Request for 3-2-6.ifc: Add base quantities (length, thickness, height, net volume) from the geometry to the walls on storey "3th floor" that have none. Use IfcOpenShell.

First a look at what the model holds.

```python
import ifcopenshell
import ifcopenshell.util.element
import ifcopenshell.util.unit

model = ifcopenshell.open("3-2-6.ifc")
print(model.schema)
for unit_type in ("LENGTHUNIT", "AREAUNIT", "VOLUMEUNIT"):
    print(unit_type, ifcopenshell.util.unit.calculate_unit_scale(model, unit_type))
storey = next(s for s in model.by_type("IfcBuildingStorey") if s.Name == "3th floor")
walls = [e for e in ifcopenshell.util.element.get_decomposition(storey) if e.is_a("IfcWall")]
for e in sorted(walls, key=lambda e: e.id()):
    print(e.id(), e.is_a(), e.Name, list(ifcopenshell.util.element.get_psets(e, qtos_only=True)), sep=" | ")
```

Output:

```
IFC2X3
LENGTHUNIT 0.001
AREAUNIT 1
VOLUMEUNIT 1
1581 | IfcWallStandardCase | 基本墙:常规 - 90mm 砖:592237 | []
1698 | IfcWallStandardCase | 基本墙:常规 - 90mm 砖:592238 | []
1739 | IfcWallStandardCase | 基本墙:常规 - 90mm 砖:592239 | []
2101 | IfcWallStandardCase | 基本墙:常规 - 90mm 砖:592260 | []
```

```python
import ifcopenshell
import ifcopenshell.api.pset
import ifcopenshell.geom
import ifcopenshell.util.element
import ifcopenshell.util.shape
import ifcopenshell.util.unit

model = ifcopenshell.open("3-2-6.ifc")
unit_scale = ifcopenshell.util.unit.calculate_unit_scale(model)
volume_scale = ifcopenshell.util.unit.calculate_unit_scale(model, "VOLUMEUNIT")
settings = ifcopenshell.geom.settings()

storey = next(s for s in model.by_type("IfcBuildingStorey") if s.Name == "3th floor")
walls = [e for e in ifcopenshell.util.element.get_decomposition(storey) if e.is_a("IfcWall")]

for e in sorted(walls, key=lambda e: e.id()):
    if ifcopenshell.util.element.get_psets(e, qtos_only=True, should_inherit=False):
        continue
    # Geometry comes back in metres, in the element's own axes.
    shape = ifcopenshell.geom.create_shape(settings, e)
    values = {
        "Length": ifcopenshell.util.shape.get_x(shape.geometry) / unit_scale,
        "Width": ifcopenshell.util.shape.get_y(shape.geometry) / unit_scale,
        "Height": ifcopenshell.util.shape.get_z(shape.geometry) / unit_scale,
        "NetVolume": ifcopenshell.util.shape.get_volume(shape.geometry) / volume_scale,
    }
    qto = ifcopenshell.api.pset.add_qto(model, product=e, name="BaseQuantities")
    ifcopenshell.api.pset.edit_qto(model, qto=qto, properties=values)
    print(e.id(), {k: round(v, 3) for k, v in values.items()})

model.write("3-2-6_edited.ifc")
```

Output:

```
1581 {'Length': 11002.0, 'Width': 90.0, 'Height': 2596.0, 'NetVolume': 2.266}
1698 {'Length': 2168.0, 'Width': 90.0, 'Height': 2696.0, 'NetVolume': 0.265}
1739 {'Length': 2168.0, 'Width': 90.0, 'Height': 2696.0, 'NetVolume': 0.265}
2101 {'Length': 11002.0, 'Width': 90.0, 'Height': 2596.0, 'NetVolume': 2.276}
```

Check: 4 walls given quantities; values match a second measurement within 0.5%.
